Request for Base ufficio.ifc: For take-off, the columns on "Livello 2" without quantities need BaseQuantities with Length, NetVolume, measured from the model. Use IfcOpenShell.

First a look at what the model holds.

```python
import ifcopenshell
import ifcopenshell.util.element
import ifcopenshell.util.unit

model = ifcopenshell.open("Base ufficio.ifc")
print(model.schema)
for unit_type in ("LENGTHUNIT", "AREAUNIT", "VOLUMEUNIT"):
    print(unit_type, ifcopenshell.util.unit.calculate_unit_scale(model, unit_type))
storey = next(s for s in model.by_type("IfcBuildingStorey") if s.Name == "Livello 2")
columns = [e for e in ifcopenshell.util.element.get_decomposition(storey) if e.is_a("IfcColumn")]
for e in sorted(columns, key=lambda e: e.id()):
    print(e.id(), e.is_a(), e.Name, list(ifcopenshell.util.element.get_psets(e, qtos_only=True)), sep=" | ")
```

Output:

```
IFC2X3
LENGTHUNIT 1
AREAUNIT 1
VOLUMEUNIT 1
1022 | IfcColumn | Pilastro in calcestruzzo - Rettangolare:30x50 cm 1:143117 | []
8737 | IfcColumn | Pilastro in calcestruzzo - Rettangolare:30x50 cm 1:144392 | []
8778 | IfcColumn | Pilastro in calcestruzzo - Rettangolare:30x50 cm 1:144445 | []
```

```python
import ifcopenshell
import ifcopenshell.api.pset
import ifcopenshell.geom
import ifcopenshell.util.element
import ifcopenshell.util.shape
import ifcopenshell.util.unit

model = ifcopenshell.open("Base ufficio.ifc")
unit_scale = ifcopenshell.util.unit.calculate_unit_scale(model)
volume_scale = ifcopenshell.util.unit.calculate_unit_scale(model, "VOLUMEUNIT")
settings = ifcopenshell.geom.settings()

storey = next(s for s in model.by_type("IfcBuildingStorey") if s.Name == "Livello 2")
columns = [e for e in ifcopenshell.util.element.get_decomposition(storey) if e.is_a("IfcColumn")]

for e in sorted(columns, key=lambda e: e.id()):
    if ifcopenshell.util.element.get_psets(e, qtos_only=True, should_inherit=False):
        continue
    # Geometry comes back in metres, in the element's own axes.
    shape = ifcopenshell.geom.create_shape(settings, e)
    values = {
        "Length": ifcopenshell.util.shape.get_z(shape.geometry) / unit_scale,
        "NetVolume": ifcopenshell.util.shape.get_volume(shape.geometry) / volume_scale,
    }
    qto = ifcopenshell.api.pset.add_qto(model, product=e, name="BaseQuantities")
    ifcopenshell.api.pset.edit_qto(model, qto=qto, properties=values)
    print(e.id(), {k: round(v, 3) for k, v in values.items()})

model.write("Base ufficio_rev.ifc")
```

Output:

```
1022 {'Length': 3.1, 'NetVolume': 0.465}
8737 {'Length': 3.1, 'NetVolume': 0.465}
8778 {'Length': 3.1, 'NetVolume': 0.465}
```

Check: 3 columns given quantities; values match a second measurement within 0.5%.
